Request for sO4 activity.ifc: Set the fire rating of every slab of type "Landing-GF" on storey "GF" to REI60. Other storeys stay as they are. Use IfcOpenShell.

First a look at what the model holds.

```python
import ifcopenshell
import ifcopenshell.util.element

model = ifcopenshell.open("sO4 activity.ifc")
print(model.schema)
storey = next(s for s in model.by_type("IfcBuildingStorey") if s.Name == "GF")
slabs = [e for e in ifcopenshell.util.element.get_decomposition(storey) if e.is_a("IfcSlab")]
seen = {}
for e in slabs:
    element_type = ifcopenshell.util.element.get_type(e)
    key = (element_type.Name if element_type != e and element_type else None, ifcopenshell.util.element.get_pset(e, "Pset_SlabCommon", "FireRating"))
    seen[key] = seen.get(key, 0) + 1
for (name, value), count in sorted(seen.items(), key=str):
    print(count, "x", name, "|", value)
```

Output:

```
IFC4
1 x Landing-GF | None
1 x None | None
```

```python
import ifcopenshell
import ifcopenshell.api.pset
import ifcopenshell.util.element

model = ifcopenshell.open("sO4 activity.ifc")

storey = next(s for s in model.by_type("IfcBuildingStorey") if s.Name == "GF")
slabs = [e for e in ifcopenshell.util.element.get_decomposition(storey) if e.is_a("IfcSlab")]

count = 0
for e in slabs:
    element_type = ifcopenshell.util.element.get_type(e)
    if element_type in (None, e) or element_type.Name != "Landing-GF":
        continue
    # add_pset returns the element's existing set when there is one.
    pset = ifcopenshell.api.pset.add_pset(model, product=e, name="Pset_SlabCommon")
    ifcopenshell.api.pset.edit_pset(model, pset=pset, properties={"FireRating": "REI60"})
    count += 1

print(count, "slabs updated")

model.write("sO4 activity_updated.ifc")
```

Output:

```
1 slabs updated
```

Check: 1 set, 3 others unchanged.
